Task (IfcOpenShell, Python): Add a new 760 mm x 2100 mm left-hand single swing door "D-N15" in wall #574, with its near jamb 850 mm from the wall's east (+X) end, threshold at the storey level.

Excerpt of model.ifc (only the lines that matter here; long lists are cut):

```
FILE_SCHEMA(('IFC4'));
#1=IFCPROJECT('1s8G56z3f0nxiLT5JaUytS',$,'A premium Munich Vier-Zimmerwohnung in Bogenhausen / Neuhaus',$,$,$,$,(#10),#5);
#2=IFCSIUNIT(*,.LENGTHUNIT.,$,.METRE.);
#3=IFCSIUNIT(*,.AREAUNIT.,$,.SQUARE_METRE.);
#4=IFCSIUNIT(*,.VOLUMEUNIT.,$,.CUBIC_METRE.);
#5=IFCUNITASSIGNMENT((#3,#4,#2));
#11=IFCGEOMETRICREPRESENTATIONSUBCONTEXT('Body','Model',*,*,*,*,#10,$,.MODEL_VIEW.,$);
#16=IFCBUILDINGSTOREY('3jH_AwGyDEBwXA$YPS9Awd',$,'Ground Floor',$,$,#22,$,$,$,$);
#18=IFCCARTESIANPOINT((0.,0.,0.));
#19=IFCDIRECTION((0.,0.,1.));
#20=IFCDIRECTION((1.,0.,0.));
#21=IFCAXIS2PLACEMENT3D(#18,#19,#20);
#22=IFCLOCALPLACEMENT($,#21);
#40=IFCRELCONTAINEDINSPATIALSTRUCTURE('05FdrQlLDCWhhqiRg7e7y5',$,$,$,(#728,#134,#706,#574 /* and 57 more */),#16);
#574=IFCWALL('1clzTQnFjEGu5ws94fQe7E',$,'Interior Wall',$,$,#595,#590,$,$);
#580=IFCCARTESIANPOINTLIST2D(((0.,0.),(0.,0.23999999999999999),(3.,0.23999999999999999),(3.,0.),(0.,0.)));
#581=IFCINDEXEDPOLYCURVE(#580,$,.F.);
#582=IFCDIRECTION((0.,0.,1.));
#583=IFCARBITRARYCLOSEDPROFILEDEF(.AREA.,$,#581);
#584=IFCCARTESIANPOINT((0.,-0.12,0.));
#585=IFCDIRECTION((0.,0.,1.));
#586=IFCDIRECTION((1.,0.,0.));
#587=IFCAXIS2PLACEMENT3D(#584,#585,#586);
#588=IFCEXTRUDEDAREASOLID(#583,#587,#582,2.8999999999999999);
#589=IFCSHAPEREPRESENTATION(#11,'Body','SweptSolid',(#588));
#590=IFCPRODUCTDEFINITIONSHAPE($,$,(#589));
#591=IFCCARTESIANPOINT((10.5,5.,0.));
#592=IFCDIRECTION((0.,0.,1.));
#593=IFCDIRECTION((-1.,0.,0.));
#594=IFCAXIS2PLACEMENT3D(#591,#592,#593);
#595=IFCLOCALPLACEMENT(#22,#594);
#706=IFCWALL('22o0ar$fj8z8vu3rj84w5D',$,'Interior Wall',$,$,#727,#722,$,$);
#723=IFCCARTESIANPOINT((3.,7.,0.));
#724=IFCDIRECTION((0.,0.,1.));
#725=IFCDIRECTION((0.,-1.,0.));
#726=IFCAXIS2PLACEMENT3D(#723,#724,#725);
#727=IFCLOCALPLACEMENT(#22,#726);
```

```python
import numpy as np
import ifcopenshell
import ifcopenshell.api.feature
import ifcopenshell.api.geometry
import ifcopenshell.api.root
import ifcopenshell.api.spatial
import ifcopenshell.geom
import ifcopenshell.util.element
import ifcopenshell.util.placement
import ifcopenshell.util.representation
import ifcopenshell.util.shape
import ifcopenshell.util.unit

model = ifcopenshell.open("model.ifc")
unit_scale = ifcopenshell.util.unit.calculate_unit_scale(model)
settings = ifcopenshell.geom.settings()


def volume(element):
    """Net volume in cubic metres, openings subtracted."""
    shape = ifcopenshell.geom.create_shape(settings, element)
    return ifcopenshell.util.shape.get_volume(shape.geometry)


wall = model.by_guid("1clzTQnFjEGu5ws94fQe7E")
storey = ifcopenshell.util.element.get_container(wall, ifc_class="IfcBuildingStorey")
context = ifcopenshell.util.representation.get_context(model, "Model", "Body", "MODEL_VIEW")
before = volume(wall)

width, height, from_end, sill = 0.76, 2.1, 0.85, 0.0  # metres

# The wall runs along its own X axis, and the end named is its -X end.
wall_shape = ifcopenshell.geom.create_shape(settings, wall)
x, y, z = ifcopenshell.util.shape.get_vertices(wall_shape.geometry).T
start = x.min() + from_end
face, thickness = float(y.min()), float(y.max() - y.min())
wall_matrix = ifcopenshell.util.placement.get_local_placement(wall.ObjectPlacement)
level = ifcopenshell.util.placement.get_local_placement(storey.ObjectPlacement)[2, 3]


def in_wall(x, y):
    """Placement at x, y metres in the wall's axes, at sill height."""
    matrix = wall_matrix.copy()
    matrix[:, 3] = wall_matrix @ np.array([x / unit_scale, y / unit_scale, 0.0, 1.0])
    matrix[2, 3] = level + sill / unit_scale
    return matrix


# Opening: a box that overshoots both wall faces by 50 mm.
opening = ifcopenshell.api.root.create_entity(model, ifc_class="IfcOpeningElement", predefined_type="OPENING")
box = ifcopenshell.api.geometry.add_wall_representation(
    model, context=context, length=width, height=height, thickness=thickness + 0.1
)
ifcopenshell.api.geometry.assign_representation(model, product=opening, representation=box)
ifcopenshell.api.geometry.edit_object_placement(model, product=opening, matrix=in_wall(start, face - 0.05), is_si=False)
ifcopenshell.api.feature.add_feature(model, feature=opening, element=wall)

door = ifcopenshell.api.root.create_entity(model, ifc_class="IfcDoor", name="D-N15", predefined_type="DOOR")
door.OverallWidth, door.OverallHeight = width / unit_scale, height / unit_scale
door.OperationType = "SINGLE_SWING_LEFT"
body = ifcopenshell.api.geometry.add_door_representation(
    model,
    context=context,
    overall_width=door.OverallWidth,
    overall_height=door.OverallHeight,
    operation_type="SINGLE_SWING_LEFT",
    lining_properties={"LiningDepth": thickness / unit_scale, "ThresholdDepth": thickness / unit_scale},
)
ifcopenshell.api.geometry.assign_representation(model, product=door, representation=body)
ifcopenshell.api.spatial.assign_container(model, products=[door], relating_structure=storey)
ifcopenshell.api.feature.add_filling(model, opening=opening, element=door)

# The lining spans the wall, so the door starts at the wall face.
ifcopenshell.api.geometry.edit_object_placement(model, product=door, matrix=in_wall(start, face), is_si=False)

after = volume(wall)

print(f"wall volume {before:.3f} -> {after:.3f} m3")

model.write("model_updated.ifc")
```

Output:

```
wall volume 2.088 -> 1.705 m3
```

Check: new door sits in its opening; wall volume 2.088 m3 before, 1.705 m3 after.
